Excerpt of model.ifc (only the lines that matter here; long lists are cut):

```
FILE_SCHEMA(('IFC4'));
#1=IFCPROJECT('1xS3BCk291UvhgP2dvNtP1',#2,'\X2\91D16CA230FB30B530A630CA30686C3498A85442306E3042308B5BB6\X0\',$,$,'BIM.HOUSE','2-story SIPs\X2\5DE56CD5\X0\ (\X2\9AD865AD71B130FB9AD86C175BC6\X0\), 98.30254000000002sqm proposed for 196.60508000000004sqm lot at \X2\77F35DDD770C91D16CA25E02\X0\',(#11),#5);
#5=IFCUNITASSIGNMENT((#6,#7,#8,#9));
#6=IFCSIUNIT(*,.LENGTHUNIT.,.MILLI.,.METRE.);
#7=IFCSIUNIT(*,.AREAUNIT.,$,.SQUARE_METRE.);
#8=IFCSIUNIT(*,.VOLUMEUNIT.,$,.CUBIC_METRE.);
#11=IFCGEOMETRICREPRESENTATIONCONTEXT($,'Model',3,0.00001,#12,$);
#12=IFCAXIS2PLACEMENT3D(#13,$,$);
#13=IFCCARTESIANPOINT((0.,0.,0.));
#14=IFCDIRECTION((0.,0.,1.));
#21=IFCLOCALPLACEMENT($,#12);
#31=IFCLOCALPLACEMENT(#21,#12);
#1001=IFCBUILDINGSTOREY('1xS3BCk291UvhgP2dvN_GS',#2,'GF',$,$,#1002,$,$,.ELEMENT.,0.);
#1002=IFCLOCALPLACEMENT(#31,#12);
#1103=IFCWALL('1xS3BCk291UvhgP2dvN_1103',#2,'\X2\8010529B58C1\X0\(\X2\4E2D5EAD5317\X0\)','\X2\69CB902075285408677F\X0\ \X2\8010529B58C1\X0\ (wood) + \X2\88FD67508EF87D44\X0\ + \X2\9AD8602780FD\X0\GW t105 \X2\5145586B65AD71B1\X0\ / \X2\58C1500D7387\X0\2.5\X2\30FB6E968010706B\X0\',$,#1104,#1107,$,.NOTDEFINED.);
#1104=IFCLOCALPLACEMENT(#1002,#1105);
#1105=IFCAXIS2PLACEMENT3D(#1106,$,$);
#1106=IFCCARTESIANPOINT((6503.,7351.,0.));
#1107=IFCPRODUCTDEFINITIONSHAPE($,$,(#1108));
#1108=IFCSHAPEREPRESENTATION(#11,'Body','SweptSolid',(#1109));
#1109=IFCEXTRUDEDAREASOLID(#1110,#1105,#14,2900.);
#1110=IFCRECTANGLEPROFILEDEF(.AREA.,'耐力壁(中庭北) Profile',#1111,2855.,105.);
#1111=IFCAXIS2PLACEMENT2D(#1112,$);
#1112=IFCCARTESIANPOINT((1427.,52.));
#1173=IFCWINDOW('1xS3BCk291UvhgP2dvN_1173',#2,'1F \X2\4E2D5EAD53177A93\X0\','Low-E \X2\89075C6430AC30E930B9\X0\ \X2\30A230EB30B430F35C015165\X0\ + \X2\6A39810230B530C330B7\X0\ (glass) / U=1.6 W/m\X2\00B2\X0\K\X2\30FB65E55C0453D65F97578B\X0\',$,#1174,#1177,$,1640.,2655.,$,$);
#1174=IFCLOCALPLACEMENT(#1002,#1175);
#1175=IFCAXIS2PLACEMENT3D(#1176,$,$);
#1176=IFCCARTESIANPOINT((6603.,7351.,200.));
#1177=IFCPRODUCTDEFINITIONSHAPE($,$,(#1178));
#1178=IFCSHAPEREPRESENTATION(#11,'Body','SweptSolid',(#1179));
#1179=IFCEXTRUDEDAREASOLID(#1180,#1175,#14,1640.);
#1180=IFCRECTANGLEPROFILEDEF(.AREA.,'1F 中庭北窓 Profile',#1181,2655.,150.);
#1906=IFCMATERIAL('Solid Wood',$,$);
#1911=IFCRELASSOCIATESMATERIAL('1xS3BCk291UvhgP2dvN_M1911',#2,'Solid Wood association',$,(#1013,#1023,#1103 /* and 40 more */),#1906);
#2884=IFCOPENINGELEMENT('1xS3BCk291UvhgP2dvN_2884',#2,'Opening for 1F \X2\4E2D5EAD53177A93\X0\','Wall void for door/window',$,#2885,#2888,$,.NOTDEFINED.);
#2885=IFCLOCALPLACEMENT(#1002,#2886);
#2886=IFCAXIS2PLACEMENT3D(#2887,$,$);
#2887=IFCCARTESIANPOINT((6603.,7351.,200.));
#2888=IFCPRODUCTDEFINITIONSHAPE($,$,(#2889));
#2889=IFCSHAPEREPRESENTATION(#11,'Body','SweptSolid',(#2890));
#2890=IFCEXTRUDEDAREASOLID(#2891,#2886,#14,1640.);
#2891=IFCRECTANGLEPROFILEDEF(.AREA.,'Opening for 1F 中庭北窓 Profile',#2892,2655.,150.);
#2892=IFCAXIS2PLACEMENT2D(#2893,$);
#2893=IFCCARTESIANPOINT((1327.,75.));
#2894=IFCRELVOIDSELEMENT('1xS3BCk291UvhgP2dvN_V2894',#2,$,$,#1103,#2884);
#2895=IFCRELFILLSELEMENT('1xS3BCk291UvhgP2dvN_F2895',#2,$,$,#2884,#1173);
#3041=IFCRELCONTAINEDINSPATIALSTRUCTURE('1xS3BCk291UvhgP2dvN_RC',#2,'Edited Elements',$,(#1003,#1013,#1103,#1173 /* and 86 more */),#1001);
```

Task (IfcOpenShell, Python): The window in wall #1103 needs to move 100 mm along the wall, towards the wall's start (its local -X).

```python
import ifcopenshell
import ifcopenshell.api.geometry
import ifcopenshell.util.placement

model = ifcopenshell.open("model.ifc")

window = model.by_guid("1xS3BCk291UvhgP2dvN_1173")
opening = window.FillsVoids[0].RelatingOpeningElement
wall = opening.VoidsElements[0].RelatingBuildingElement

wall_matrix = ifcopenshell.util.placement.get_local_placement(wall.ObjectPlacement)
shift = wall_matrix[:3, 0] * -100.0
before = ifcopenshell.util.placement.get_local_placement(window.ObjectPlacement)[:3, 3].copy()

# The window is not placed relative to its opening, so move both.
for product in (opening, window):
    matrix = ifcopenshell.util.placement.get_local_placement(product.ObjectPlacement)
    matrix[:3, 3] += shift
    ifcopenshell.api.geometry.edit_object_placement(model, product=product, matrix=matrix, is_si=False)

after = ifcopenshell.util.placement.get_local_placement(window.ObjectPlacement)[:3, 3]
print("window moved by", (after - before).round(3) + 0.0)

model.write("model_updated.ifc")
```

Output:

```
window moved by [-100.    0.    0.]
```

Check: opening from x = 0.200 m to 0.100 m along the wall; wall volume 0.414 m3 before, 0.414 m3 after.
